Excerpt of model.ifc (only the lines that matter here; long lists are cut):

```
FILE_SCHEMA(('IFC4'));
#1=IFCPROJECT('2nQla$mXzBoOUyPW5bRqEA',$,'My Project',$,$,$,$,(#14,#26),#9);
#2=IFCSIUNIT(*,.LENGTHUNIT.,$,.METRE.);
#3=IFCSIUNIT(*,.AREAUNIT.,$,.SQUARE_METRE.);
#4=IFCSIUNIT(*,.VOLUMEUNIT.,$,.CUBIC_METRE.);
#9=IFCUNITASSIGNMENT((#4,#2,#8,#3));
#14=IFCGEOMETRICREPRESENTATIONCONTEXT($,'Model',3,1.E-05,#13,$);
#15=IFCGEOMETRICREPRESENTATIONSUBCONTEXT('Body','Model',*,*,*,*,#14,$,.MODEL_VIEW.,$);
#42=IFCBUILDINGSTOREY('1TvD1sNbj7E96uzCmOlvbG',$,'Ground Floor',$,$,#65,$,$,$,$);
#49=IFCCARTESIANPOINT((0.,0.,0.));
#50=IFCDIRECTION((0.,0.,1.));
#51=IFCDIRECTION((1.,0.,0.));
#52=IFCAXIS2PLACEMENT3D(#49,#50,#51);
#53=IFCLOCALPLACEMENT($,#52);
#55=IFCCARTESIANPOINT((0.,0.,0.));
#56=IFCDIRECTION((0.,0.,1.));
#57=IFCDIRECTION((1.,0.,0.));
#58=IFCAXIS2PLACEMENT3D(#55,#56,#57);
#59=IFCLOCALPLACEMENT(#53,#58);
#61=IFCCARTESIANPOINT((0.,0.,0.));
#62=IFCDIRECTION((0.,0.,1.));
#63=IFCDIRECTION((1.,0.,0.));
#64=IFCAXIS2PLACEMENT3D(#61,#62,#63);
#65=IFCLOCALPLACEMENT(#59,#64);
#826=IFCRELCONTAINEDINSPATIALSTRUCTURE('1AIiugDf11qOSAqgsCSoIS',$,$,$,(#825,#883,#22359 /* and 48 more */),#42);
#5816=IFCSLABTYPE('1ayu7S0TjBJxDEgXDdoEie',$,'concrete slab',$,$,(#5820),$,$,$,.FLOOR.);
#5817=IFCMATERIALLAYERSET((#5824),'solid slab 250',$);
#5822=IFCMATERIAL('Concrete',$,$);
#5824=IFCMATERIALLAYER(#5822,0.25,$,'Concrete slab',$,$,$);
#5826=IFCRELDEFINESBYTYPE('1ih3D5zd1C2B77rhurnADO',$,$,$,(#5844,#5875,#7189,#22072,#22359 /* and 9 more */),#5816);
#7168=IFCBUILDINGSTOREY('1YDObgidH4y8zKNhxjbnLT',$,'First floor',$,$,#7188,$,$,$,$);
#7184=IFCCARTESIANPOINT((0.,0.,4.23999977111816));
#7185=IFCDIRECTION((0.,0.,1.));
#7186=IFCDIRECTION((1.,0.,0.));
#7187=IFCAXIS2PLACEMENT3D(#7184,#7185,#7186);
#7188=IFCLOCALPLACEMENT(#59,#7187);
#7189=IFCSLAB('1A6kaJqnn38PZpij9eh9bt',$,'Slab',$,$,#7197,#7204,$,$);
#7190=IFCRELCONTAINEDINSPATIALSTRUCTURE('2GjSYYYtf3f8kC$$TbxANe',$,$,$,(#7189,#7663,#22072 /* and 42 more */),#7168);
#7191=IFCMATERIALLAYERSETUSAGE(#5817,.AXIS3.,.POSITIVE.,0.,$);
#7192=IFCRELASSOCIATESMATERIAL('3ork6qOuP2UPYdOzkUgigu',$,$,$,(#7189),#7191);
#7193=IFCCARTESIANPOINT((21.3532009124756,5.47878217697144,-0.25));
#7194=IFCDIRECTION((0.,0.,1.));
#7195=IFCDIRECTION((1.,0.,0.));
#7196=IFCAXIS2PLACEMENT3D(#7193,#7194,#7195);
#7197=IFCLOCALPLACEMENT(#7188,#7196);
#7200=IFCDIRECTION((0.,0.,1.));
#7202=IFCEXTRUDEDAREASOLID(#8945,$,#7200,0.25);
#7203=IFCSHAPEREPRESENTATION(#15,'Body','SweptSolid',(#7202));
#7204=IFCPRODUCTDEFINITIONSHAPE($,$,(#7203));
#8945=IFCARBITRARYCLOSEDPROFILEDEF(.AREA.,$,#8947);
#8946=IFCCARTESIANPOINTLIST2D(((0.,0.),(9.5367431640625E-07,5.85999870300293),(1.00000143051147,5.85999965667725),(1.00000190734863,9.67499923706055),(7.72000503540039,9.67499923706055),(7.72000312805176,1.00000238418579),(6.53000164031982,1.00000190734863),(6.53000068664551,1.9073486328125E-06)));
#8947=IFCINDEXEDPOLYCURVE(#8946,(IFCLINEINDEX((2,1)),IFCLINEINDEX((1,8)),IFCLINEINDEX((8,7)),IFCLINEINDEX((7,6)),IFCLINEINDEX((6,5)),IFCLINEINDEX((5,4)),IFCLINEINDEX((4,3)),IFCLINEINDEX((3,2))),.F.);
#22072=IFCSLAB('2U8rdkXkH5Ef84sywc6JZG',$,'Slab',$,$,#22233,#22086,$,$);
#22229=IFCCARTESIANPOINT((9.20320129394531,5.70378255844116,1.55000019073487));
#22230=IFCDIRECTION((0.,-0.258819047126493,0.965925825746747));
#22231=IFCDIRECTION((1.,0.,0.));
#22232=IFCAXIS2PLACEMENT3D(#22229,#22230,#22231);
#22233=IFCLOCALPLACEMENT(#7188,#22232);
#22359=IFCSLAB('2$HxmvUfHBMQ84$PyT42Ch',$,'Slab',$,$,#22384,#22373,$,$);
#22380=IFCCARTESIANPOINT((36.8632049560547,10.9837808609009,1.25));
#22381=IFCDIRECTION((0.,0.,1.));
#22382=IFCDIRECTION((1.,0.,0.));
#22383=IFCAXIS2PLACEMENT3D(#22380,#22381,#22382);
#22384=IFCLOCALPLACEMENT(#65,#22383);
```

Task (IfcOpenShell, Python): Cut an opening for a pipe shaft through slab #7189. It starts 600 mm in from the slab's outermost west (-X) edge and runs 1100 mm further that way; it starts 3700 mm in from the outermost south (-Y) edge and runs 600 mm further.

```python
import numpy as np
import ifcopenshell
import ifcopenshell.api.feature
import ifcopenshell.api.geometry
import ifcopenshell.api.root
import ifcopenshell.geom
import ifcopenshell.util.placement
import ifcopenshell.util.representation
import ifcopenshell.util.shape
import ifcopenshell.util.unit

model = ifcopenshell.open("model.ifc")
unit_scale = ifcopenshell.util.unit.calculate_unit_scale(model)
settings = ifcopenshell.geom.settings()


def volume(element):
    """Net volume in cubic metres, openings subtracted."""
    shape = ifcopenshell.geom.create_shape(settings, element)
    return ifcopenshell.util.shape.get_volume(shape.geometry)


slab = model.by_guid("1A6kaJqnn38PZpij9eh9bt")
before = volume(slab)

# Extent in the slab's own axes, in metres. The edges named are its -X and -Y sides.
slab_shape = ifcopenshell.geom.create_shape(settings, slab)
vertices = ifcopenshell.util.shape.get_vertices(slab_shape.geometry)
x_min, y_min, bottom = vertices.min(axis=0)
top = vertices[:, 2].max()

opening = ifcopenshell.api.root.create_entity(model, ifc_class="IfcOpeningElement", name="Pipe shaft opening", predefined_type="OPENING")
context = ifcopenshell.util.representation.get_context(model, "Model", "Body", "MODEL_VIEW")
width, depth = 1.1, 0.6
outline = [(0.0, 0.0), (width, 0.0), (width, depth), (0.0, depth), (0.0, 0.0)]
# Overshoot both faces by 50 mm so the cut is clean.
shape = ifcopenshell.api.geometry.add_slab_representation(
    model, context=context, depth=top - bottom + 0.1, polyline=outline
)
ifcopenshell.api.geometry.assign_representation(model, product=opening, representation=shape)

matrix = ifcopenshell.util.placement.get_local_placement(slab.ObjectPlacement)
matrix[:, 3] = matrix @ np.append(np.array([x_min + 0.6, y_min + 3.7, bottom - 0.05]) / unit_scale, 1.0)
ifcopenshell.api.geometry.edit_object_placement(model, product=opening, matrix=matrix, is_si=False)
ifcopenshell.api.feature.add_feature(model, feature=opening, element=slab)

after = volume(slab)

print(f"slab volume {before:.3f} -> {after:.3f} m3")

model.write("model_v2.ifc")
```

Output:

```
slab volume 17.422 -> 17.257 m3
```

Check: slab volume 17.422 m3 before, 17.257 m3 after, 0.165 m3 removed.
